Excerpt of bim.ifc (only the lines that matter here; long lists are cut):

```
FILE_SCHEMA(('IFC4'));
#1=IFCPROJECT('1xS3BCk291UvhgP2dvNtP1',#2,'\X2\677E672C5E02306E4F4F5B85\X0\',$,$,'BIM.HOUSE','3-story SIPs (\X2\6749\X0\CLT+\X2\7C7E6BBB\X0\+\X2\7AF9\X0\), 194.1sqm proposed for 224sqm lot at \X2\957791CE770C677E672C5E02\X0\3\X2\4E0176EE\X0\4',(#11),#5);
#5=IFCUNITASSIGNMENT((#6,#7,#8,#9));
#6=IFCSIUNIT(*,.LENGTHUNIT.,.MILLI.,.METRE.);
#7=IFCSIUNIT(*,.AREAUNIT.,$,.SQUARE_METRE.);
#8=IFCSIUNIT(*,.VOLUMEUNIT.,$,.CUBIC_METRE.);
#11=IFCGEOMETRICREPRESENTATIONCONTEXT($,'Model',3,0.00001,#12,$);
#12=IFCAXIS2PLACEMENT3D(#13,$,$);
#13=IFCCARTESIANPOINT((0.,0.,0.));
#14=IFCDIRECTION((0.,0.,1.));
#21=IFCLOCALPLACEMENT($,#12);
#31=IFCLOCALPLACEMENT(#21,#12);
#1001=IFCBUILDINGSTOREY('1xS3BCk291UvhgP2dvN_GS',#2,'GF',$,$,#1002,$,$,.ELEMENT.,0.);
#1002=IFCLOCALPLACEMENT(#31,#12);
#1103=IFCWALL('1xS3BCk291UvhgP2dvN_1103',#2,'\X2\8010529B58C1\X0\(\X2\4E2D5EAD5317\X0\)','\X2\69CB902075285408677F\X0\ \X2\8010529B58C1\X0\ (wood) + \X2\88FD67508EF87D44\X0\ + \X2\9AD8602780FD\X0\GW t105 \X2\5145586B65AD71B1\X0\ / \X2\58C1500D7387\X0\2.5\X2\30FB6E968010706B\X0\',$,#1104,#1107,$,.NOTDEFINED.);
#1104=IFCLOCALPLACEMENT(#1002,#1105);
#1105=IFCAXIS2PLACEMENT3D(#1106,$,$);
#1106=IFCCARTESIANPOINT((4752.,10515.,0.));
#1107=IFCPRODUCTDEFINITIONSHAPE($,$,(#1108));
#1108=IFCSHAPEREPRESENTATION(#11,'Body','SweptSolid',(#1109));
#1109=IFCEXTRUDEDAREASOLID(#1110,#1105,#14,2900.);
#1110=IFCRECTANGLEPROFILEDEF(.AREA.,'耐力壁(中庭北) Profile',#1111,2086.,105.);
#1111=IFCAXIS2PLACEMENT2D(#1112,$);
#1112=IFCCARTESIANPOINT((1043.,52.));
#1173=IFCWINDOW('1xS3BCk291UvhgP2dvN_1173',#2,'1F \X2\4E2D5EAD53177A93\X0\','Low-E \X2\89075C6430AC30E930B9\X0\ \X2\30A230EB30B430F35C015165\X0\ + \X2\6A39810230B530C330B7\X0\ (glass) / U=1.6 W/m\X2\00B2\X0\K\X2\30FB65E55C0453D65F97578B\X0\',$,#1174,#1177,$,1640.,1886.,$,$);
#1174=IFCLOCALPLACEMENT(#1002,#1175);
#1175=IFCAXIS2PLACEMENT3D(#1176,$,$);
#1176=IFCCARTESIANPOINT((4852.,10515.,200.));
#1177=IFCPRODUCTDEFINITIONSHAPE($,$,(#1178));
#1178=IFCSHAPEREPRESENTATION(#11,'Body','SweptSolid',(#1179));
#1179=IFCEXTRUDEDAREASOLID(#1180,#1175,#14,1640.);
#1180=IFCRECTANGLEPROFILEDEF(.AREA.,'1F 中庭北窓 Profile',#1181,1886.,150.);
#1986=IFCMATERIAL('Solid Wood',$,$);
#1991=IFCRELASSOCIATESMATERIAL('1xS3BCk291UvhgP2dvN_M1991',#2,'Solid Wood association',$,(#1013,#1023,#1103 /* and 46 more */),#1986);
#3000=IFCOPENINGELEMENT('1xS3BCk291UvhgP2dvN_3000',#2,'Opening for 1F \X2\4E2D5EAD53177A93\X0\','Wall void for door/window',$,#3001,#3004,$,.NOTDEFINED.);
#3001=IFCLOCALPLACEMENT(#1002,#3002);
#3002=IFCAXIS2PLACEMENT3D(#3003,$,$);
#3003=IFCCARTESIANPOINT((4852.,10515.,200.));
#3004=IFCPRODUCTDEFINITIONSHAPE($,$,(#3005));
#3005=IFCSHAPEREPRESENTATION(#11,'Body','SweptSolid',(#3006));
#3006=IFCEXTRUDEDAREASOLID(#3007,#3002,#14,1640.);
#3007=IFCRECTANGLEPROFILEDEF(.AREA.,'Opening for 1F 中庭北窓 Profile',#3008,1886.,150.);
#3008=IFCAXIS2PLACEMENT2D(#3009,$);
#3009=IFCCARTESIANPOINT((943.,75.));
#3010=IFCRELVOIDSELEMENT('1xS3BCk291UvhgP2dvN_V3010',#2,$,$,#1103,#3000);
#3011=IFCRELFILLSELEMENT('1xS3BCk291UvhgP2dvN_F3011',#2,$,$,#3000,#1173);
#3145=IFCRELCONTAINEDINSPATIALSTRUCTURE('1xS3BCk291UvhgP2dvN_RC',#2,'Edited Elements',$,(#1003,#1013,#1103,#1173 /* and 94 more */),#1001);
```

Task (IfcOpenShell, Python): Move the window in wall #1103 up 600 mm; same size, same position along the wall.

```python
import numpy as np
import ifcopenshell
import ifcopenshell.api.geometry
import ifcopenshell.util.placement
import ifcopenshell.util.unit

model = ifcopenshell.open("bim.ifc")
unit_scale = ifcopenshell.util.unit.calculate_unit_scale(model)

window = model.by_guid("1xS3BCk291UvhgP2dvN_1173")
opening = window.FillsVoids[0].RelatingOpeningElement
dz = 600.0

shift = np.array([0.0, 0.0, dz])
# The window is not placed relative to its opening, so move both.
for product in (opening, window):
    matrix = ifcopenshell.util.placement.get_local_placement(product.ObjectPlacement)
    matrix[:3, 3] += shift
    ifcopenshell.api.geometry.edit_object_placement(model, product=product, matrix=matrix, is_si=False)

print(f"moved by {dz * unit_scale:+.3f} m")

model.write("bim-out.ifc")
```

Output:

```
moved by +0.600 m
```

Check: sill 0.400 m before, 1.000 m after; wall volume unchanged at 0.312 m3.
